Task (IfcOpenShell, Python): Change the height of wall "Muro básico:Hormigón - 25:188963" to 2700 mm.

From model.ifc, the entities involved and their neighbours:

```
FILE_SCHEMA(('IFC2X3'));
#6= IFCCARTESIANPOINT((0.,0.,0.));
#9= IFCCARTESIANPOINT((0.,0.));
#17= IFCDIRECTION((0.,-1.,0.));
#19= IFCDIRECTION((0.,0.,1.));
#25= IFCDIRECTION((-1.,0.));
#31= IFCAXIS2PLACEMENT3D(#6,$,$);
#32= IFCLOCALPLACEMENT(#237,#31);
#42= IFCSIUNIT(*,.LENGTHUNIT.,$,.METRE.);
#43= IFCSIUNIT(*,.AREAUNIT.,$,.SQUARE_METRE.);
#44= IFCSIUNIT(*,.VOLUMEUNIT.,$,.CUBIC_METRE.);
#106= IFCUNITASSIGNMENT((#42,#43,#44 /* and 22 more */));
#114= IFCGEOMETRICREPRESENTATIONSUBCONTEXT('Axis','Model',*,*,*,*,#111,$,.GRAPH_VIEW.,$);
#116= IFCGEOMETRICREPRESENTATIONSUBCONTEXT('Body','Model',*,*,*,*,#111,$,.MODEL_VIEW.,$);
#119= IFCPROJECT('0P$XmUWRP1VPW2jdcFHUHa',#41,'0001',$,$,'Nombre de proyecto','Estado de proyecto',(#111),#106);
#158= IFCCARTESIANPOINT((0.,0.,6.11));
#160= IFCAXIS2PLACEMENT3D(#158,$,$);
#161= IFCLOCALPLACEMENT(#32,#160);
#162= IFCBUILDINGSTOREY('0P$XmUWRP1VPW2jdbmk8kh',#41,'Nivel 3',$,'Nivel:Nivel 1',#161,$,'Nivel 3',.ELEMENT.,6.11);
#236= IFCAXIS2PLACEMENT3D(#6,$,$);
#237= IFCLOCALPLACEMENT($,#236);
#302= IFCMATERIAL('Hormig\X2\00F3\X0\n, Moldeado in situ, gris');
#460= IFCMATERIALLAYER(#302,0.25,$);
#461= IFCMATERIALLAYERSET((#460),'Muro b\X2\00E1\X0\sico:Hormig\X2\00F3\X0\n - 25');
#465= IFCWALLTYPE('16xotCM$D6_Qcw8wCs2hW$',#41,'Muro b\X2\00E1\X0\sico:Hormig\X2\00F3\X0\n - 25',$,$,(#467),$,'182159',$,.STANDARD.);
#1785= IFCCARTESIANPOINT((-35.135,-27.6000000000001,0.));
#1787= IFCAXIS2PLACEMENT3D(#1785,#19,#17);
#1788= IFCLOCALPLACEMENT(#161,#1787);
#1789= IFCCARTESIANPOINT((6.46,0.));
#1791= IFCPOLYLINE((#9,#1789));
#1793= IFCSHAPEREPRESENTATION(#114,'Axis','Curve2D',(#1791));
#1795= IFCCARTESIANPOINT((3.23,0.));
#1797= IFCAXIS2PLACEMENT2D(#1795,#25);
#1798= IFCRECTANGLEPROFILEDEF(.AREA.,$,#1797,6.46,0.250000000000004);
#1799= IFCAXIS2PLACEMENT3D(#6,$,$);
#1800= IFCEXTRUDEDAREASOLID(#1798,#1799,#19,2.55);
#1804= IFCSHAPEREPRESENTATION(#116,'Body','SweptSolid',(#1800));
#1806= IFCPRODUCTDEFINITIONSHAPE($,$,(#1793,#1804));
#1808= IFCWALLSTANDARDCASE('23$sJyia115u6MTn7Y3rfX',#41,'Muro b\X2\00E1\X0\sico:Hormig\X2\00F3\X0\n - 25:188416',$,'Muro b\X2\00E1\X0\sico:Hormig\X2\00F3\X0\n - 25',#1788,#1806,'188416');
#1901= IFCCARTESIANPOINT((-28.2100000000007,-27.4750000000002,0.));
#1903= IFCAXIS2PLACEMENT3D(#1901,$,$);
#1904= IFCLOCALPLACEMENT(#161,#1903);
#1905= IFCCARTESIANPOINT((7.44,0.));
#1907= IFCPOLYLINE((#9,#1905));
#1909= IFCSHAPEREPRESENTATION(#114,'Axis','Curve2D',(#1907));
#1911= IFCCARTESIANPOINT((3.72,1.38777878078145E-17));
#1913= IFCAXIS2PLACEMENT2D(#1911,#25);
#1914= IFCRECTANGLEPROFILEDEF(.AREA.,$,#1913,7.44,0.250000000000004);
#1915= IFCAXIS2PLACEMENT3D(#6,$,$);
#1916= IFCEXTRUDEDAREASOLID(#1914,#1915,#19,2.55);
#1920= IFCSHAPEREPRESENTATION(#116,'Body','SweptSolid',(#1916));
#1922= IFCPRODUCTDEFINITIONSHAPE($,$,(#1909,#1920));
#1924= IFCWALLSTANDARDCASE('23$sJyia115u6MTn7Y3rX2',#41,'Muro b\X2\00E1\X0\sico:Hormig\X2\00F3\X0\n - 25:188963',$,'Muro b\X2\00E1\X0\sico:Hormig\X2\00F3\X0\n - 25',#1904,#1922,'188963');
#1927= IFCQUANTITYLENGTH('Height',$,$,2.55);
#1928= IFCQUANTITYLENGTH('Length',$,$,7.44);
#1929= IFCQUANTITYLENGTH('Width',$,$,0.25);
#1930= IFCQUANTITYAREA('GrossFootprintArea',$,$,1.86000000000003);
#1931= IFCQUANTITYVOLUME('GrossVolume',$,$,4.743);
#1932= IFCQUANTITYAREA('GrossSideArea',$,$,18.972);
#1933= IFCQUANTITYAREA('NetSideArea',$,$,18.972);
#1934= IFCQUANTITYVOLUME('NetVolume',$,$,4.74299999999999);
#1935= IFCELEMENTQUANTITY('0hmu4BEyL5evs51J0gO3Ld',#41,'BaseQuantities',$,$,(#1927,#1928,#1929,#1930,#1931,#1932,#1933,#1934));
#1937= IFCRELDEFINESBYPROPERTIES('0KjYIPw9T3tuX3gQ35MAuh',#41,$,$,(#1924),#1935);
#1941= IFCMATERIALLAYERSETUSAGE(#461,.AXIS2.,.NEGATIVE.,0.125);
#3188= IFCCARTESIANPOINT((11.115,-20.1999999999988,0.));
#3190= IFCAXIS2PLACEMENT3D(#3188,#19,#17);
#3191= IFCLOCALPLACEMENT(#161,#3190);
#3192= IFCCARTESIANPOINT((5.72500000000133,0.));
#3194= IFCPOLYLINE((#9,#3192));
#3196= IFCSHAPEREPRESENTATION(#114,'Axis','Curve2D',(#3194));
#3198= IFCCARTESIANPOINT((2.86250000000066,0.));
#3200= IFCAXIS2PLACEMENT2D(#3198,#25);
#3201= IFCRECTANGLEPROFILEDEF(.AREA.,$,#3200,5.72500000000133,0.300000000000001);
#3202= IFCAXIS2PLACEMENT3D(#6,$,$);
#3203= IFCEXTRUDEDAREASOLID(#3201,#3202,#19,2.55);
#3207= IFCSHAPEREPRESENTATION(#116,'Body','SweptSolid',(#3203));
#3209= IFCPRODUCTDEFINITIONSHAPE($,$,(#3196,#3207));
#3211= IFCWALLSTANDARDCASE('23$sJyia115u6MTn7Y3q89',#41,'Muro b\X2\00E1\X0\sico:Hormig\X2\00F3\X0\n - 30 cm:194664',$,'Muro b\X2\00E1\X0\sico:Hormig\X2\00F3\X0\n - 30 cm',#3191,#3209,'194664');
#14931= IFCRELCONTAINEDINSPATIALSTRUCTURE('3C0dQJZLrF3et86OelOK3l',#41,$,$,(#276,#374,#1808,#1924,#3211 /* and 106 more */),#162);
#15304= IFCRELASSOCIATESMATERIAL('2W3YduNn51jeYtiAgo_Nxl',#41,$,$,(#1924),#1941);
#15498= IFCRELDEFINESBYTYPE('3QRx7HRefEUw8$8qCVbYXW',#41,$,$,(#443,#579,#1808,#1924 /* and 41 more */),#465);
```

```python
import ifcopenshell
import ifcopenshell.api.pset
import ifcopenshell.geom
import ifcopenshell.util.element
import ifcopenshell.util.representation
import ifcopenshell.util.shape
import ifcopenshell.util.unit

model = ifcopenshell.open("model.ifc")
unit_scale = ifcopenshell.util.unit.calculate_unit_scale(model)
area_scale = ifcopenshell.util.unit.calculate_unit_scale(model, "AREAUNIT")
volume_scale = ifcopenshell.util.unit.calculate_unit_scale(model, "VOLUMEUNIT")
settings = ifcopenshell.geom.settings()


def volume(element):
    """Net volume in cubic metres, openings subtracted."""
    shape = ifcopenshell.geom.create_shape(settings, element)
    return ifcopenshell.util.shape.get_volume(shape.geometry)


wall = model.by_id(1924)
before = volume(wall)

body = ifcopenshell.util.representation.get_representation(wall, "Model", "Body")
solid = body.Items[0]
old_height = solid.Depth
solid.Depth = 2.7 / unit_scale
after = volume(wall)
thickness = 0.25  # wall thickness in metres

# Update the stored height, areas and volumes.
qto = model.by_id(ifcopenshell.util.element.get_pset(wall, "BaseQuantities", should_inherit=False)["id"])
ifcopenshell.api.pset.edit_qto(model, qto=qto, properties={
    "Height": solid.Depth,
    "GrossVolume": ifcopenshell.util.element.get_pset(wall, "BaseQuantities", "GrossVolume") * solid.Depth / old_height,
    "GrossSideArea": ifcopenshell.util.element.get_pset(wall, "BaseQuantities", "GrossSideArea") * solid.Depth / old_height,
    "NetSideArea": after / thickness / area_scale,
    "NetVolume": after / volume_scale,
})

print(f"height {old_height:g} -> {solid.Depth:g}, volume {before:.3f} -> {after:.3f} m3")

model.write("model-out.ifc")
```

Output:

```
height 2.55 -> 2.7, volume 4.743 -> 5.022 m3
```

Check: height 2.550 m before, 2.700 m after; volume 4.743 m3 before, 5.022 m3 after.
